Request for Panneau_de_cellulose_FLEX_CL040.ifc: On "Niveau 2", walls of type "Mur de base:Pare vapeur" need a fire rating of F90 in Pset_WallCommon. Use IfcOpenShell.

First a look at what the model holds.

```python
import ifcopenshell
import ifcopenshell.util.element

model = ifcopenshell.open("Panneau_de_cellulose_FLEX_CL040.ifc")
print(model.schema)
storey = next(s for s in model.by_type("IfcBuildingStorey") if s.Name == "Niveau 2")
walls = [e for e in ifcopenshell.util.element.get_decomposition(storey) if e.is_a("IfcWall")]
seen = {}
for e in walls:
    element_type = ifcopenshell.util.element.get_type(e)
    key = (element_type.Name if element_type != e and element_type else None, ifcopenshell.util.element.get_pset(e, "Pset_WallCommon", "FireRating"))
    seen[key] = seen.get(key, 0) + 1
for (name, value), count in sorted(seen.items(), key=str):
    print(count, "x", name, "|", value)
```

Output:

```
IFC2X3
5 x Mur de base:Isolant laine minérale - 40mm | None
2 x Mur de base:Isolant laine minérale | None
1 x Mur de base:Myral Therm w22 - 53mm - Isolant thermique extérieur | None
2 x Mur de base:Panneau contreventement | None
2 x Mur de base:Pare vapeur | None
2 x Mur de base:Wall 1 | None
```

```python
import ifcopenshell
import ifcopenshell.api.pset
import ifcopenshell.util.element

model = ifcopenshell.open("Panneau_de_cellulose_FLEX_CL040.ifc")

storey = next(s for s in model.by_type("IfcBuildingStorey") if s.Name == "Niveau 2")
walls = [e for e in ifcopenshell.util.element.get_decomposition(storey) if e.is_a("IfcWall")]

count = 0
for e in walls:
    element_type = ifcopenshell.util.element.get_type(e)
    if element_type in (None, e) or element_type.Name != "Mur de base:Pare vapeur":
        continue
    # add_pset returns the element's existing set when there is one.
    pset = ifcopenshell.api.pset.add_pset(model, product=e, name="Pset_WallCommon")
    ifcopenshell.api.pset.edit_pset(model, pset=pset, properties={"FireRating": "F90"})
    count += 1

print(count, "walls updated")

model.write("Panneau_de_cellulose_FLEX_CL040_edited.ifc")
```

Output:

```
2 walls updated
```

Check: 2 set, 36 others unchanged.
